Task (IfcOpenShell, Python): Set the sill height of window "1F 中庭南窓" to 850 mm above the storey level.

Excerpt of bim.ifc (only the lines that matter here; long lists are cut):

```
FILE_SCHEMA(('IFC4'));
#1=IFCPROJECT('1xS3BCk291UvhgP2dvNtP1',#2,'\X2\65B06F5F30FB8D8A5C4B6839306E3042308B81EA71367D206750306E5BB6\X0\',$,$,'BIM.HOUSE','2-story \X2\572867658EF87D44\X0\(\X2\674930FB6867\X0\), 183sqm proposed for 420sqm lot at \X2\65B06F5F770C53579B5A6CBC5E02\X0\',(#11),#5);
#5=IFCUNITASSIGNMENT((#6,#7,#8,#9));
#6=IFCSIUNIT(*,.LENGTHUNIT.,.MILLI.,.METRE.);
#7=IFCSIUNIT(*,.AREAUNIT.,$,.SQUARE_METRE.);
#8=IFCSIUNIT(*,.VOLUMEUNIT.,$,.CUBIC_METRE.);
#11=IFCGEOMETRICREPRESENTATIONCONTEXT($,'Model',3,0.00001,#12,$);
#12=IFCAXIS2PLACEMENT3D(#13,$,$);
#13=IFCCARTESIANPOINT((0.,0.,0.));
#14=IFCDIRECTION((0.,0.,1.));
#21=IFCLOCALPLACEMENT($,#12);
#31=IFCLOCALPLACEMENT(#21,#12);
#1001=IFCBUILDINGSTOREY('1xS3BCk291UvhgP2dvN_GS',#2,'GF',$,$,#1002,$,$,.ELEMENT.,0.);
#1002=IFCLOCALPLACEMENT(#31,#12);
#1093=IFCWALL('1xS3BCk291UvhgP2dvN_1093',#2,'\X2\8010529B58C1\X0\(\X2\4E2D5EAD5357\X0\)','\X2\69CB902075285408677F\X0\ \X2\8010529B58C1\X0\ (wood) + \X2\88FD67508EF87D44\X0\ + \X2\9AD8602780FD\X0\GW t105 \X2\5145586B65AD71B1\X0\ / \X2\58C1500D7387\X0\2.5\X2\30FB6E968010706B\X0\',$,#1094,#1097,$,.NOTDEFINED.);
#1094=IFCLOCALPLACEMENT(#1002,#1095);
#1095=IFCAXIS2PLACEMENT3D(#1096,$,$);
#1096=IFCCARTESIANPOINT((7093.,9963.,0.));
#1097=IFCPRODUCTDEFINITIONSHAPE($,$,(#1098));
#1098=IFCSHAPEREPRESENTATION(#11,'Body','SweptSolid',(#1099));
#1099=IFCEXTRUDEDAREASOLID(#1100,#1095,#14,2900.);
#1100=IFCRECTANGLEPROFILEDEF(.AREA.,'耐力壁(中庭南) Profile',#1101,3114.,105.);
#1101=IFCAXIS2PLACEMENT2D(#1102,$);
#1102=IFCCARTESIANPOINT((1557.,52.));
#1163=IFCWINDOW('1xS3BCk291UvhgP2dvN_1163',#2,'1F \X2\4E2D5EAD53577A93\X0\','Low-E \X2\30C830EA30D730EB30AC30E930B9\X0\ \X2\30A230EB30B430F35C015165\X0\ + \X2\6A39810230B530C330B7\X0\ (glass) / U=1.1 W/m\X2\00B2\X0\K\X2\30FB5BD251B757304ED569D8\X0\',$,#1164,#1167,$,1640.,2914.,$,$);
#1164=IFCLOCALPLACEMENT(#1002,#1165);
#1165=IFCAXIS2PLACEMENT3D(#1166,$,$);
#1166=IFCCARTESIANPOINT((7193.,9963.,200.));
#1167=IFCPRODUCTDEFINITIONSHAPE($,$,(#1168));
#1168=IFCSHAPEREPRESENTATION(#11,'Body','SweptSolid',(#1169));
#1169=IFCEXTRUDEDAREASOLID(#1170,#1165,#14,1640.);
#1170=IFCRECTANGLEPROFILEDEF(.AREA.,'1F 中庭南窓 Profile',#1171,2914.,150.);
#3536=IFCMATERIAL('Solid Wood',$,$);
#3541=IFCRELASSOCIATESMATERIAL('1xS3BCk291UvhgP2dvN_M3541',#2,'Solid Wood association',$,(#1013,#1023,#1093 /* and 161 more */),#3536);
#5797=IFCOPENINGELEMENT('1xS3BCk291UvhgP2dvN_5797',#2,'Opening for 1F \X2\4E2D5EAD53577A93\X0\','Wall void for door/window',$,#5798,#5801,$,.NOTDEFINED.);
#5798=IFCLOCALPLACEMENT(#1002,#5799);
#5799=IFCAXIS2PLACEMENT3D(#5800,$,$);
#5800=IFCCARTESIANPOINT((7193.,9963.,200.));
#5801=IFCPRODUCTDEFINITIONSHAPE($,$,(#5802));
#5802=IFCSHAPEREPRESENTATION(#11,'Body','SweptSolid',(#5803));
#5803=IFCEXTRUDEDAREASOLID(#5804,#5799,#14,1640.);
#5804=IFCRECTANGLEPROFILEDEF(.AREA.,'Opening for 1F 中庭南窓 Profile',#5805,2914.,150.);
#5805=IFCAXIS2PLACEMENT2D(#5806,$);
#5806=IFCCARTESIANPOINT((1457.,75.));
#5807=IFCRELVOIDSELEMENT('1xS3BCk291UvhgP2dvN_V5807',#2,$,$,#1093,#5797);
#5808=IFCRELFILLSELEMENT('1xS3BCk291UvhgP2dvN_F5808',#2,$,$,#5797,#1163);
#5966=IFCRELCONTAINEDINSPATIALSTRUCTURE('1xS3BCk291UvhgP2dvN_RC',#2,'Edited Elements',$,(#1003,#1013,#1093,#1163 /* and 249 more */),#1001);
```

```python
import numpy as np
import ifcopenshell
import ifcopenshell.api.geometry
import ifcopenshell.geom
import ifcopenshell.util.element
import ifcopenshell.util.placement
import ifcopenshell.util.shape
import ifcopenshell.util.unit

model = ifcopenshell.open("bim.ifc")
unit_scale = ifcopenshell.util.unit.calculate_unit_scale(model)

window = model.by_guid("1xS3BCk291UvhgP2dvN_1163")
opening = window.FillsVoids[0].RelatingOpeningElement
storey = ifcopenshell.util.element.get_container(window, ifc_class="IfcBuildingStorey")
level = ifcopenshell.util.placement.get_local_placement(storey.ObjectPlacement)[2, 3]

# The opening's origin need not be at the sill, so measure its lowest point.
shape = ifcopenshell.geom.create_shape(ifcopenshell.geom.settings(), opening)
bottom = ifcopenshell.util.shape.get_shape_bottom_elevation(shape, shape.geometry) / unit_scale
dz = level + 850.0 - bottom

shift = np.array([0.0, 0.0, dz])
# The window is not placed relative to its opening, so move both.
for product in (opening, window):
    matrix = ifcopenshell.util.placement.get_local_placement(product.ObjectPlacement)
    matrix[:3, 3] += shift
    ifcopenshell.api.geometry.edit_object_placement(model, product=product, matrix=matrix, is_si=False)

print(f"moved by {dz * unit_scale:+.3f} m")

model.write("bim-out.ifc")
```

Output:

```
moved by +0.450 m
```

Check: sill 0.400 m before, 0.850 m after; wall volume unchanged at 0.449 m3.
